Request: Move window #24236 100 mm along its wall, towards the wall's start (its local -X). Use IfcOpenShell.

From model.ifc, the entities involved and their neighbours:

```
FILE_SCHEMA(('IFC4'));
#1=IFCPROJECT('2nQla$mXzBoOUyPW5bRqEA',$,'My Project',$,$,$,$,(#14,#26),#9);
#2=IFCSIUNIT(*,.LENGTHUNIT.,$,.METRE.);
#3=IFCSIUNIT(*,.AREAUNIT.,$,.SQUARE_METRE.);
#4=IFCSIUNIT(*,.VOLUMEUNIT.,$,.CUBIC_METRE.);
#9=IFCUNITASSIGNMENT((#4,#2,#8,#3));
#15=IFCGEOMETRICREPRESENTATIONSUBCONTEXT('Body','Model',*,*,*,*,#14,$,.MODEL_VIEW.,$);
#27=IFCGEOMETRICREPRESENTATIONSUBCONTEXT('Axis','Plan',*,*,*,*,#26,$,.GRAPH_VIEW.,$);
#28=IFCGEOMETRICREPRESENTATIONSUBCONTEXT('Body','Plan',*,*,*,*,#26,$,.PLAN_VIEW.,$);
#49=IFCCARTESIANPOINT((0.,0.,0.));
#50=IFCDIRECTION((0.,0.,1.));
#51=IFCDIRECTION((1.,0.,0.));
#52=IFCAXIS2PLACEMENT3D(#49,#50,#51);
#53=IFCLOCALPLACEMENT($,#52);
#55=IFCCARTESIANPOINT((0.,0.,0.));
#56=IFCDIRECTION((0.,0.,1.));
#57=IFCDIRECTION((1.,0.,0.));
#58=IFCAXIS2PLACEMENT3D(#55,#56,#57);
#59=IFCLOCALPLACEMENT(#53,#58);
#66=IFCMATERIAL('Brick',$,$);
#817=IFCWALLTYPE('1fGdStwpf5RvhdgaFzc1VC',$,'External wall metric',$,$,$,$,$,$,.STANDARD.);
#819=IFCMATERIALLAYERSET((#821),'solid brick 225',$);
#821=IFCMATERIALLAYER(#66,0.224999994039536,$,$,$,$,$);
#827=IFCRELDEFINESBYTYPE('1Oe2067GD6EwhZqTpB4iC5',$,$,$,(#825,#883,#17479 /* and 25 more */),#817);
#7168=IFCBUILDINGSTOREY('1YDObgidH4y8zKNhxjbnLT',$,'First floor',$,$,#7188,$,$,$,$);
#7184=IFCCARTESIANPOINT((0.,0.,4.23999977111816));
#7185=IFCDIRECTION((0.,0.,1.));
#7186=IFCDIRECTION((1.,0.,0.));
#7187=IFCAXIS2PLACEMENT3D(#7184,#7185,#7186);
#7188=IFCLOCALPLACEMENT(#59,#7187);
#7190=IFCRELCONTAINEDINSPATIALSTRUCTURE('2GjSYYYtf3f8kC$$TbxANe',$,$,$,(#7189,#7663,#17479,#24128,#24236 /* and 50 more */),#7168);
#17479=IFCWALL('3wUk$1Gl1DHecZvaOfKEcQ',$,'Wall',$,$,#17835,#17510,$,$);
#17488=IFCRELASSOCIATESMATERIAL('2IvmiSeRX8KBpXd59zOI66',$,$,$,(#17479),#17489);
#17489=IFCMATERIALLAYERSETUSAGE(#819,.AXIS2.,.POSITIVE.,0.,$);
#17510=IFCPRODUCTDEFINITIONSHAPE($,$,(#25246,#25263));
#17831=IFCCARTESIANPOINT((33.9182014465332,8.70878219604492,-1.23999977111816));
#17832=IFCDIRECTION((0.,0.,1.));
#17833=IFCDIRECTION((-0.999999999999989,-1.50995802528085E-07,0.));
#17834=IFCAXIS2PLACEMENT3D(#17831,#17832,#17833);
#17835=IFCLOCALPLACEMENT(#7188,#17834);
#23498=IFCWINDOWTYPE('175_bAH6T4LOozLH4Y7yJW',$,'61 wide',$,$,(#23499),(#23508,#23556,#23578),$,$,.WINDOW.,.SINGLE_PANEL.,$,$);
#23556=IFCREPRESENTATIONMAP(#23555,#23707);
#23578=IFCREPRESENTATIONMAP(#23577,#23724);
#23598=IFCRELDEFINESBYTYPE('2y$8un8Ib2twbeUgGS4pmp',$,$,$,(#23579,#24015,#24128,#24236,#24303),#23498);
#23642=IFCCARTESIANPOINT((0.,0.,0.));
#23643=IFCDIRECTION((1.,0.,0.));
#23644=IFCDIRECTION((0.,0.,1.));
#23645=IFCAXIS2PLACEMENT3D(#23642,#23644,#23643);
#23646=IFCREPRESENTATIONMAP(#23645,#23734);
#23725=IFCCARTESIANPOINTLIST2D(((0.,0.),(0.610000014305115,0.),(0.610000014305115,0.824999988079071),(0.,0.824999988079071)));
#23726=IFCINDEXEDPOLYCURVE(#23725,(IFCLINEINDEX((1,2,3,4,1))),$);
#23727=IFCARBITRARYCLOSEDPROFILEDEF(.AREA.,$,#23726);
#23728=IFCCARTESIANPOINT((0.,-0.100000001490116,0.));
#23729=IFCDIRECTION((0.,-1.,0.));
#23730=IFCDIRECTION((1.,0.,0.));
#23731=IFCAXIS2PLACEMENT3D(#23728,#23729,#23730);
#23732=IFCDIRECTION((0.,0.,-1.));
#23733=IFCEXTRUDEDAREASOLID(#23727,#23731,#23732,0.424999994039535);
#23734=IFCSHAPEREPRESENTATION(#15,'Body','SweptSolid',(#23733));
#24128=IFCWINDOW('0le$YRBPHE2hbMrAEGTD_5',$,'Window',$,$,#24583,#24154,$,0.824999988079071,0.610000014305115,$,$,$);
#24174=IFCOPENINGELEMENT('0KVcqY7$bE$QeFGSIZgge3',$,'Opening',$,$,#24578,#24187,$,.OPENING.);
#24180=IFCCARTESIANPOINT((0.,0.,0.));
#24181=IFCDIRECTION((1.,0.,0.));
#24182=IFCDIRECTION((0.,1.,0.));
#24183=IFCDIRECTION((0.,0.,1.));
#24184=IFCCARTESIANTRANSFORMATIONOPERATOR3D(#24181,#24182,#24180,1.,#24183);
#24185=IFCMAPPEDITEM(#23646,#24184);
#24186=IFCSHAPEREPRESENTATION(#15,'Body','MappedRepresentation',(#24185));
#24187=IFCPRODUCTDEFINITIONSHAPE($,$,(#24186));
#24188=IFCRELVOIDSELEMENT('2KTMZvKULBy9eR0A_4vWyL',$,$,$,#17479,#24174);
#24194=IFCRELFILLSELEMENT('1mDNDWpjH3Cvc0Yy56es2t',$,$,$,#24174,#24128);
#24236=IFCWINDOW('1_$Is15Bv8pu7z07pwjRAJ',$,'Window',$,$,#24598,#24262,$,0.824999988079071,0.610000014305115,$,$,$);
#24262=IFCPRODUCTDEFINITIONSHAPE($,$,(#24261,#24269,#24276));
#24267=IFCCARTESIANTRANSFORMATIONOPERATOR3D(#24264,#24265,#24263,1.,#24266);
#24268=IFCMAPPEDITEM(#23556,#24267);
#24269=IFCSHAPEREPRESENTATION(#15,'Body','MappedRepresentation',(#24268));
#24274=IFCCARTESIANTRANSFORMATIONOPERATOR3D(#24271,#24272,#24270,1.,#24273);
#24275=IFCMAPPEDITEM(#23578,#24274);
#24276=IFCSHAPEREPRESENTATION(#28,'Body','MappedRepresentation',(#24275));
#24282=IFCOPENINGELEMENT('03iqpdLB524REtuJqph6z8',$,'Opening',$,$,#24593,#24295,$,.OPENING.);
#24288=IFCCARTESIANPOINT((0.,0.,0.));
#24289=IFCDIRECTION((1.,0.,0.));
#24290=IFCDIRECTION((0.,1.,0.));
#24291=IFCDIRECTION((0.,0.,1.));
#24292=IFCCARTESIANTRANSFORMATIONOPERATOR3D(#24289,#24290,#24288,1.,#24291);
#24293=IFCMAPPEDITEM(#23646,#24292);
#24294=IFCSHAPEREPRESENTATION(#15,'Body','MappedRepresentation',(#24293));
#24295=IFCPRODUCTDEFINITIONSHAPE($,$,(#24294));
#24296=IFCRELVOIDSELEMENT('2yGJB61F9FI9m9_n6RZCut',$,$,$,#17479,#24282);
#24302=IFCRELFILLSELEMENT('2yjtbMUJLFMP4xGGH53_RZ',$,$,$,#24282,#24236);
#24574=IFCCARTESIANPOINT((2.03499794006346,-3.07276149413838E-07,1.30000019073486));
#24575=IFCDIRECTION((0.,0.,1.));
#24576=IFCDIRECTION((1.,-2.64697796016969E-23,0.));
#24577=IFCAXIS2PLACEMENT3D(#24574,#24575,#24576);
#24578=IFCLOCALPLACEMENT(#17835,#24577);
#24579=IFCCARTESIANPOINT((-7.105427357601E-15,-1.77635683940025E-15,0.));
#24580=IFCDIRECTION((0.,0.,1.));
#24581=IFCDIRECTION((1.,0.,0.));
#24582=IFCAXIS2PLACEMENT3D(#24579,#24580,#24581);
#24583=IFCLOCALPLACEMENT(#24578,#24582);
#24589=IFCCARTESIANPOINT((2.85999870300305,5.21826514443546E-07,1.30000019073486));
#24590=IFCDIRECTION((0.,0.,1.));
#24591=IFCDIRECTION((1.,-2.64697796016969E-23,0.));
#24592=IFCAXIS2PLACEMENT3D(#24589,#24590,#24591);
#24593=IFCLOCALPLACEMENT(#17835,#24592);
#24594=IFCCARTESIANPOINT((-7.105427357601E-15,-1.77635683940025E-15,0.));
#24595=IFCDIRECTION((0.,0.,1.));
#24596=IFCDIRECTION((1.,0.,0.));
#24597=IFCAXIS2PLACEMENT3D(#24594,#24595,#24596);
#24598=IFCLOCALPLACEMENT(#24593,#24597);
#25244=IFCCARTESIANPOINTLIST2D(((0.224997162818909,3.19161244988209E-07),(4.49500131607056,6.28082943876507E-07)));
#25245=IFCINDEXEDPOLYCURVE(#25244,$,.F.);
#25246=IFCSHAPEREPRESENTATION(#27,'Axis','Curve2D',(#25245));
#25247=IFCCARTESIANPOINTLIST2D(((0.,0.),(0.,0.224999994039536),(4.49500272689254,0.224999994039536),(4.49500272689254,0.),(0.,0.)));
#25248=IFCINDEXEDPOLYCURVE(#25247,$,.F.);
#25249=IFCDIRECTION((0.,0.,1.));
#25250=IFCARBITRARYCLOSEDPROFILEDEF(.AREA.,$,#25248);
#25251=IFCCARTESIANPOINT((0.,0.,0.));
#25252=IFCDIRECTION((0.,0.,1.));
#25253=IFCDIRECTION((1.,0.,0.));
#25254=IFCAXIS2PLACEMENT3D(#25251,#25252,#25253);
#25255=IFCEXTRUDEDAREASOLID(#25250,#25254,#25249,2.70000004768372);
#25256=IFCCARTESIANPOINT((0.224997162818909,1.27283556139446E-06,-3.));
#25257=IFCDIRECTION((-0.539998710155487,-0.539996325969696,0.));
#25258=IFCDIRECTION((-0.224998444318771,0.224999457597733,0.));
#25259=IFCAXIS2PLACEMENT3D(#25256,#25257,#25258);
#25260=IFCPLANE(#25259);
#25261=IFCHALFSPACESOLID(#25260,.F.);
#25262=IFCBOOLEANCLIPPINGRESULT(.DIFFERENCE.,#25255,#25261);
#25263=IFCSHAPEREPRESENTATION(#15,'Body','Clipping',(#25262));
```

```python
import ifcopenshell
import ifcopenshell.api.geometry
import ifcopenshell.util.placement
import ifcopenshell.util.unit

model = ifcopenshell.open("model.ifc")
unit_scale = ifcopenshell.util.unit.calculate_unit_scale(model)

window = model.by_guid("1_$Is15Bv8pu7z07pwjRAJ")
opening = window.FillsVoids[0].RelatingOpeningElement
wall = opening.VoidsElements[0].RelatingBuildingElement

wall_matrix = ifcopenshell.util.placement.get_local_placement(wall.ObjectPlacement)
shift = wall_matrix[:3, 0] * -0.1 / unit_scale
before = ifcopenshell.util.placement.get_local_placement(window.ObjectPlacement)[:3, 3].copy()

# The window is placed relative to its opening, so it follows when the opening moves.
matrix = ifcopenshell.util.placement.get_local_placement(opening.ObjectPlacement)
matrix[:3, 3] += shift
ifcopenshell.api.geometry.edit_object_placement(
    model, product=opening, matrix=matrix, is_si=False, should_transform_children=True
)

after = ifcopenshell.util.placement.get_local_placement(window.ObjectPlacement)[:3, 3]
print("window moved by", (after - before).round(3) + 0.0)

model.write("model_v2.ifc")
```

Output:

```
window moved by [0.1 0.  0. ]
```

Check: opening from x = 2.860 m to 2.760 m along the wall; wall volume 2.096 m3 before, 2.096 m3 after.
